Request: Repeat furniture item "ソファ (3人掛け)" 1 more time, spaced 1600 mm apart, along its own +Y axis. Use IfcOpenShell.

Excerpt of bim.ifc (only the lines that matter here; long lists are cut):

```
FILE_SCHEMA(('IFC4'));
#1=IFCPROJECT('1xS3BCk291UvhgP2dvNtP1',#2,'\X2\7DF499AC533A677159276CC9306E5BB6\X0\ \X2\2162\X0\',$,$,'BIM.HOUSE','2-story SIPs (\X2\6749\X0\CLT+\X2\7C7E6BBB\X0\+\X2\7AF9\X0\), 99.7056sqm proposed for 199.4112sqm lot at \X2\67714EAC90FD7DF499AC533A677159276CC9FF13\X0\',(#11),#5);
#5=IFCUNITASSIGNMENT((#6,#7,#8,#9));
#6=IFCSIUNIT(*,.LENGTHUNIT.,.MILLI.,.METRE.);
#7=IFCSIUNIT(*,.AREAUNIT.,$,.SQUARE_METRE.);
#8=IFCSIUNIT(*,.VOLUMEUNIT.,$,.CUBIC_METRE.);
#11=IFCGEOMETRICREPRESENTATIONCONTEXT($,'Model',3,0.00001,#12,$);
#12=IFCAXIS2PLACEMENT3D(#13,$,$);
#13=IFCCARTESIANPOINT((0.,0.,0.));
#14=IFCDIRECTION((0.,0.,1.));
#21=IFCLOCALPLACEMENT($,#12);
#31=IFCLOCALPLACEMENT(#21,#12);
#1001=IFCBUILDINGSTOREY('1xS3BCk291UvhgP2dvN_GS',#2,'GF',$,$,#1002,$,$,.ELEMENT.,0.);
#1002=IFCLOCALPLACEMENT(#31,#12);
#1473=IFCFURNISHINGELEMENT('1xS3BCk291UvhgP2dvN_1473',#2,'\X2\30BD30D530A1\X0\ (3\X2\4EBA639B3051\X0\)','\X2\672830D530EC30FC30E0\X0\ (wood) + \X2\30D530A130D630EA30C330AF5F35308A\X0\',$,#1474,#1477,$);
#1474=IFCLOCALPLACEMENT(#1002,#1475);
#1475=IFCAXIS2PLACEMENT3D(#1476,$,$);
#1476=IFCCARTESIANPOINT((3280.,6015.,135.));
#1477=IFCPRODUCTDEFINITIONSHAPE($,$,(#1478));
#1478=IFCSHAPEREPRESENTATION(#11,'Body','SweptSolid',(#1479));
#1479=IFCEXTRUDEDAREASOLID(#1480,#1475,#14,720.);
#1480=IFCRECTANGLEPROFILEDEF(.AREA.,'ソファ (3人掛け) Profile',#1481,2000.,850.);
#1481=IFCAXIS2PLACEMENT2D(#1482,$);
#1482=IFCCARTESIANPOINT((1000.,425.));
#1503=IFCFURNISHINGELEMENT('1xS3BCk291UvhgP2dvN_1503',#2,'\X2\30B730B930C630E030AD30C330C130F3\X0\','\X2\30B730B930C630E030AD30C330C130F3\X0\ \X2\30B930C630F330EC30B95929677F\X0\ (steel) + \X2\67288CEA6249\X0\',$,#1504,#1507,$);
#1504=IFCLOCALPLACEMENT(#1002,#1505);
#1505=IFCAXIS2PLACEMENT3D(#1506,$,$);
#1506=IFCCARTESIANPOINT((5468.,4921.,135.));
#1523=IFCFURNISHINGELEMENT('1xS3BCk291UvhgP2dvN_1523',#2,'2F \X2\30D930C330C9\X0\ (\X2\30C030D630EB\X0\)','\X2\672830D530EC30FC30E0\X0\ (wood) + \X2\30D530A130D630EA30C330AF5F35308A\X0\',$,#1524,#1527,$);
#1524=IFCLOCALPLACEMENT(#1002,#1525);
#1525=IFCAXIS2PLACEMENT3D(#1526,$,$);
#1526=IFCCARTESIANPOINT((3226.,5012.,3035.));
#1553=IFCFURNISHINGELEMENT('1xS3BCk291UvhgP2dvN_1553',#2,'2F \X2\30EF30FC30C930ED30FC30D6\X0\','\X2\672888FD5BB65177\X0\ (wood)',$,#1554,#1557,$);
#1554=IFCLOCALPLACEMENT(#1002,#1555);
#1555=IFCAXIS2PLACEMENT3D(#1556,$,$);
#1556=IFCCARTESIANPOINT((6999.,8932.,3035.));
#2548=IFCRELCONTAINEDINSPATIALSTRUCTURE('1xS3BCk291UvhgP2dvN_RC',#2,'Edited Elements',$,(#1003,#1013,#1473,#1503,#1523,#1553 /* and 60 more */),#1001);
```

```python
import ifcopenshell
import ifcopenshell.api.geometry
import ifcopenshell.api.root
import ifcopenshell.util.element
import ifcopenshell.util.placement
import ifcopenshell.util.unit

model = ifcopenshell.open("bim.ifc")
unit_scale = ifcopenshell.util.unit.calculate_unit_scale(model)


def reuse_history(source, copy):
    """copy_class also copies each property set's owner history, people and application; keep the originals."""
    for rel in copy.IsDefinedBy:
        if rel.is_a("IfcRelDefinesByProperties") and (history := rel.RelatingPropertyDefinition.OwnerHistory):
            rel.RelatingPropertyDefinition.OwnerHistory = source.OwnerHistory
            ifcopenshell.util.element.remove_deep2(model, history)


source = model.by_id(1473)
base = ifcopenshell.util.placement.get_local_placement(source.ObjectPlacement)
step = base[:3, 1] * 1.6 / unit_scale

for i in range(1, 2):
    copy = ifcopenshell.api.root.copy_class(model, product=source)
    copy.Representation = ifcopenshell.util.element.copy_deep(
        model, source.Representation, exclude=["IfcGeometricRepresentationContext", "IfcRepresentationMap"]
    )
    reuse_history(source, copy)
    matrix = base.copy()
    matrix[:3, 3] += i * step
    print("added at", matrix[:3, 3].round(3) + 0.0)
    ifcopenshell.api.geometry.edit_object_placement(model, product=copy, matrix=matrix, is_si=False)

model.write("bim_updated.ifc")
```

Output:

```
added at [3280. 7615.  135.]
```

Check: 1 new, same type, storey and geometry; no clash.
